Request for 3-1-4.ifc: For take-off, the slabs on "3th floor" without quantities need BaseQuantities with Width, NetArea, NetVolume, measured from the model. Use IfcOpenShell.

First a look at what the model holds.

```python
import ifcopenshell
import ifcopenshell.util.element
import ifcopenshell.util.unit

model = ifcopenshell.open("3-1-4.ifc")
print(model.schema)
for unit_type in ("LENGTHUNIT", "AREAUNIT", "VOLUMEUNIT"):
    print(unit_type, ifcopenshell.util.unit.calculate_unit_scale(model, unit_type))
storey = next(s for s in model.by_type("IfcBuildingStorey") if s.Name == "3th floor")
slabs = [e for e in ifcopenshell.util.element.get_decomposition(storey) if e.is_a("IfcSlab")]
for e in sorted(slabs, key=lambda e: e.id()):
    print(e.id(), e.is_a(), e.Name, list(ifcopenshell.util.element.get_psets(e, qtos_only=True)), sep=" | ")
```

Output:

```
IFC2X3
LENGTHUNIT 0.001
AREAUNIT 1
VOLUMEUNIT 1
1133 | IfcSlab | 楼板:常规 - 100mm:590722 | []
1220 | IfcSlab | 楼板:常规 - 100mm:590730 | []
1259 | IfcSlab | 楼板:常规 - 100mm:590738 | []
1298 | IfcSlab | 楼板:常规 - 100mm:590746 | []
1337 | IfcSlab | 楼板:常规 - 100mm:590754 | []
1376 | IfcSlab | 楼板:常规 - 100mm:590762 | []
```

```python
import ifcopenshell
import ifcopenshell.api.pset
import ifcopenshell.geom
import ifcopenshell.util.element
import ifcopenshell.util.shape
import ifcopenshell.util.unit

model = ifcopenshell.open("3-1-4.ifc")
unit_scale = ifcopenshell.util.unit.calculate_unit_scale(model)
area_scale = ifcopenshell.util.unit.calculate_unit_scale(model, "AREAUNIT")
volume_scale = ifcopenshell.util.unit.calculate_unit_scale(model, "VOLUMEUNIT")
settings = ifcopenshell.geom.settings()

storey = next(s for s in model.by_type("IfcBuildingStorey") if s.Name == "3th floor")
slabs = [e for e in ifcopenshell.util.element.get_decomposition(storey) if e.is_a("IfcSlab")]

for e in sorted(slabs, key=lambda e: e.id()):
    if ifcopenshell.util.element.get_psets(e, qtos_only=True, should_inherit=False):
        continue
    # Geometry comes back in metres, in the element's own axes.
    shape = ifcopenshell.geom.create_shape(settings, e)
    values = {
        "Width": ifcopenshell.util.shape.get_z(shape.geometry) / unit_scale,
        "NetArea": ifcopenshell.util.shape.get_footprint_area(shape.geometry) / area_scale,
        "NetVolume": ifcopenshell.util.shape.get_volume(shape.geometry) / volume_scale,
    }
    qto = ifcopenshell.api.pset.add_qto(model, product=e, name="BaseQuantities")
    ifcopenshell.api.pset.edit_qto(model, qto=qto, properties=values)
    print(e.id(), {k: round(v, 3) for k, v in values.items()})

model.write("3-1-4_edited.ifc")
```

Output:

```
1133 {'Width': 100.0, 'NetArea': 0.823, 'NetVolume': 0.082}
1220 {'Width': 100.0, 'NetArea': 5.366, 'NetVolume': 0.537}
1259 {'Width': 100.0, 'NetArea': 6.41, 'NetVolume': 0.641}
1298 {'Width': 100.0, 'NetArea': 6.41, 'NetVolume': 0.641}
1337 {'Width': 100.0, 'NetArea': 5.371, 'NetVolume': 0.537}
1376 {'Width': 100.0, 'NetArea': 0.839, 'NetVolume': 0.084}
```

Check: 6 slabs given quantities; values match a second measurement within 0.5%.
